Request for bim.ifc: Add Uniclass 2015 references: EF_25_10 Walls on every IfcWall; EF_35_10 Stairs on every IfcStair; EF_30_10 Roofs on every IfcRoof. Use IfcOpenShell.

First a look at what the model holds.

```python
import ifcopenshell

model = ifcopenshell.open("bim.ifc")
print(model.schema)
print("classifications:", [c.Name for c in model.by_type("IfcClassification")])
for ifc_class in ("IfcDoor", "IfcRoof", "IfcStair", "IfcWall", "IfcWindow"):
    print(ifc_class, len(model.by_type(ifc_class)))
```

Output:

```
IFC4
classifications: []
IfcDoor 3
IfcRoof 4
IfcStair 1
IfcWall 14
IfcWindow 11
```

```python
import ifcopenshell
import ifcopenshell.api.classification

model = ifcopenshell.open("bim.ifc")

system = ifcopenshell.api.classification.add_classification(model, classification="Uniclass 2015")

codes = {
    "IfcWall": ("EF_25_10", "Walls"),
    "IfcStair": ("EF_35_10", "Stairs"),
    "IfcRoof": ("EF_30_10", "Roofs"),
}
for ifc_class, (code, name) in codes.items():
    products = model.by_type(ifc_class)
    ifcopenshell.api.classification.add_reference(
        model, products=products, classification=system, identification=code, name=name
    )
    print(code, len(products))

model.write("bim_rev.ifc")
```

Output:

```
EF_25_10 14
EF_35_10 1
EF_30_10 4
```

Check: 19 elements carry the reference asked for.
